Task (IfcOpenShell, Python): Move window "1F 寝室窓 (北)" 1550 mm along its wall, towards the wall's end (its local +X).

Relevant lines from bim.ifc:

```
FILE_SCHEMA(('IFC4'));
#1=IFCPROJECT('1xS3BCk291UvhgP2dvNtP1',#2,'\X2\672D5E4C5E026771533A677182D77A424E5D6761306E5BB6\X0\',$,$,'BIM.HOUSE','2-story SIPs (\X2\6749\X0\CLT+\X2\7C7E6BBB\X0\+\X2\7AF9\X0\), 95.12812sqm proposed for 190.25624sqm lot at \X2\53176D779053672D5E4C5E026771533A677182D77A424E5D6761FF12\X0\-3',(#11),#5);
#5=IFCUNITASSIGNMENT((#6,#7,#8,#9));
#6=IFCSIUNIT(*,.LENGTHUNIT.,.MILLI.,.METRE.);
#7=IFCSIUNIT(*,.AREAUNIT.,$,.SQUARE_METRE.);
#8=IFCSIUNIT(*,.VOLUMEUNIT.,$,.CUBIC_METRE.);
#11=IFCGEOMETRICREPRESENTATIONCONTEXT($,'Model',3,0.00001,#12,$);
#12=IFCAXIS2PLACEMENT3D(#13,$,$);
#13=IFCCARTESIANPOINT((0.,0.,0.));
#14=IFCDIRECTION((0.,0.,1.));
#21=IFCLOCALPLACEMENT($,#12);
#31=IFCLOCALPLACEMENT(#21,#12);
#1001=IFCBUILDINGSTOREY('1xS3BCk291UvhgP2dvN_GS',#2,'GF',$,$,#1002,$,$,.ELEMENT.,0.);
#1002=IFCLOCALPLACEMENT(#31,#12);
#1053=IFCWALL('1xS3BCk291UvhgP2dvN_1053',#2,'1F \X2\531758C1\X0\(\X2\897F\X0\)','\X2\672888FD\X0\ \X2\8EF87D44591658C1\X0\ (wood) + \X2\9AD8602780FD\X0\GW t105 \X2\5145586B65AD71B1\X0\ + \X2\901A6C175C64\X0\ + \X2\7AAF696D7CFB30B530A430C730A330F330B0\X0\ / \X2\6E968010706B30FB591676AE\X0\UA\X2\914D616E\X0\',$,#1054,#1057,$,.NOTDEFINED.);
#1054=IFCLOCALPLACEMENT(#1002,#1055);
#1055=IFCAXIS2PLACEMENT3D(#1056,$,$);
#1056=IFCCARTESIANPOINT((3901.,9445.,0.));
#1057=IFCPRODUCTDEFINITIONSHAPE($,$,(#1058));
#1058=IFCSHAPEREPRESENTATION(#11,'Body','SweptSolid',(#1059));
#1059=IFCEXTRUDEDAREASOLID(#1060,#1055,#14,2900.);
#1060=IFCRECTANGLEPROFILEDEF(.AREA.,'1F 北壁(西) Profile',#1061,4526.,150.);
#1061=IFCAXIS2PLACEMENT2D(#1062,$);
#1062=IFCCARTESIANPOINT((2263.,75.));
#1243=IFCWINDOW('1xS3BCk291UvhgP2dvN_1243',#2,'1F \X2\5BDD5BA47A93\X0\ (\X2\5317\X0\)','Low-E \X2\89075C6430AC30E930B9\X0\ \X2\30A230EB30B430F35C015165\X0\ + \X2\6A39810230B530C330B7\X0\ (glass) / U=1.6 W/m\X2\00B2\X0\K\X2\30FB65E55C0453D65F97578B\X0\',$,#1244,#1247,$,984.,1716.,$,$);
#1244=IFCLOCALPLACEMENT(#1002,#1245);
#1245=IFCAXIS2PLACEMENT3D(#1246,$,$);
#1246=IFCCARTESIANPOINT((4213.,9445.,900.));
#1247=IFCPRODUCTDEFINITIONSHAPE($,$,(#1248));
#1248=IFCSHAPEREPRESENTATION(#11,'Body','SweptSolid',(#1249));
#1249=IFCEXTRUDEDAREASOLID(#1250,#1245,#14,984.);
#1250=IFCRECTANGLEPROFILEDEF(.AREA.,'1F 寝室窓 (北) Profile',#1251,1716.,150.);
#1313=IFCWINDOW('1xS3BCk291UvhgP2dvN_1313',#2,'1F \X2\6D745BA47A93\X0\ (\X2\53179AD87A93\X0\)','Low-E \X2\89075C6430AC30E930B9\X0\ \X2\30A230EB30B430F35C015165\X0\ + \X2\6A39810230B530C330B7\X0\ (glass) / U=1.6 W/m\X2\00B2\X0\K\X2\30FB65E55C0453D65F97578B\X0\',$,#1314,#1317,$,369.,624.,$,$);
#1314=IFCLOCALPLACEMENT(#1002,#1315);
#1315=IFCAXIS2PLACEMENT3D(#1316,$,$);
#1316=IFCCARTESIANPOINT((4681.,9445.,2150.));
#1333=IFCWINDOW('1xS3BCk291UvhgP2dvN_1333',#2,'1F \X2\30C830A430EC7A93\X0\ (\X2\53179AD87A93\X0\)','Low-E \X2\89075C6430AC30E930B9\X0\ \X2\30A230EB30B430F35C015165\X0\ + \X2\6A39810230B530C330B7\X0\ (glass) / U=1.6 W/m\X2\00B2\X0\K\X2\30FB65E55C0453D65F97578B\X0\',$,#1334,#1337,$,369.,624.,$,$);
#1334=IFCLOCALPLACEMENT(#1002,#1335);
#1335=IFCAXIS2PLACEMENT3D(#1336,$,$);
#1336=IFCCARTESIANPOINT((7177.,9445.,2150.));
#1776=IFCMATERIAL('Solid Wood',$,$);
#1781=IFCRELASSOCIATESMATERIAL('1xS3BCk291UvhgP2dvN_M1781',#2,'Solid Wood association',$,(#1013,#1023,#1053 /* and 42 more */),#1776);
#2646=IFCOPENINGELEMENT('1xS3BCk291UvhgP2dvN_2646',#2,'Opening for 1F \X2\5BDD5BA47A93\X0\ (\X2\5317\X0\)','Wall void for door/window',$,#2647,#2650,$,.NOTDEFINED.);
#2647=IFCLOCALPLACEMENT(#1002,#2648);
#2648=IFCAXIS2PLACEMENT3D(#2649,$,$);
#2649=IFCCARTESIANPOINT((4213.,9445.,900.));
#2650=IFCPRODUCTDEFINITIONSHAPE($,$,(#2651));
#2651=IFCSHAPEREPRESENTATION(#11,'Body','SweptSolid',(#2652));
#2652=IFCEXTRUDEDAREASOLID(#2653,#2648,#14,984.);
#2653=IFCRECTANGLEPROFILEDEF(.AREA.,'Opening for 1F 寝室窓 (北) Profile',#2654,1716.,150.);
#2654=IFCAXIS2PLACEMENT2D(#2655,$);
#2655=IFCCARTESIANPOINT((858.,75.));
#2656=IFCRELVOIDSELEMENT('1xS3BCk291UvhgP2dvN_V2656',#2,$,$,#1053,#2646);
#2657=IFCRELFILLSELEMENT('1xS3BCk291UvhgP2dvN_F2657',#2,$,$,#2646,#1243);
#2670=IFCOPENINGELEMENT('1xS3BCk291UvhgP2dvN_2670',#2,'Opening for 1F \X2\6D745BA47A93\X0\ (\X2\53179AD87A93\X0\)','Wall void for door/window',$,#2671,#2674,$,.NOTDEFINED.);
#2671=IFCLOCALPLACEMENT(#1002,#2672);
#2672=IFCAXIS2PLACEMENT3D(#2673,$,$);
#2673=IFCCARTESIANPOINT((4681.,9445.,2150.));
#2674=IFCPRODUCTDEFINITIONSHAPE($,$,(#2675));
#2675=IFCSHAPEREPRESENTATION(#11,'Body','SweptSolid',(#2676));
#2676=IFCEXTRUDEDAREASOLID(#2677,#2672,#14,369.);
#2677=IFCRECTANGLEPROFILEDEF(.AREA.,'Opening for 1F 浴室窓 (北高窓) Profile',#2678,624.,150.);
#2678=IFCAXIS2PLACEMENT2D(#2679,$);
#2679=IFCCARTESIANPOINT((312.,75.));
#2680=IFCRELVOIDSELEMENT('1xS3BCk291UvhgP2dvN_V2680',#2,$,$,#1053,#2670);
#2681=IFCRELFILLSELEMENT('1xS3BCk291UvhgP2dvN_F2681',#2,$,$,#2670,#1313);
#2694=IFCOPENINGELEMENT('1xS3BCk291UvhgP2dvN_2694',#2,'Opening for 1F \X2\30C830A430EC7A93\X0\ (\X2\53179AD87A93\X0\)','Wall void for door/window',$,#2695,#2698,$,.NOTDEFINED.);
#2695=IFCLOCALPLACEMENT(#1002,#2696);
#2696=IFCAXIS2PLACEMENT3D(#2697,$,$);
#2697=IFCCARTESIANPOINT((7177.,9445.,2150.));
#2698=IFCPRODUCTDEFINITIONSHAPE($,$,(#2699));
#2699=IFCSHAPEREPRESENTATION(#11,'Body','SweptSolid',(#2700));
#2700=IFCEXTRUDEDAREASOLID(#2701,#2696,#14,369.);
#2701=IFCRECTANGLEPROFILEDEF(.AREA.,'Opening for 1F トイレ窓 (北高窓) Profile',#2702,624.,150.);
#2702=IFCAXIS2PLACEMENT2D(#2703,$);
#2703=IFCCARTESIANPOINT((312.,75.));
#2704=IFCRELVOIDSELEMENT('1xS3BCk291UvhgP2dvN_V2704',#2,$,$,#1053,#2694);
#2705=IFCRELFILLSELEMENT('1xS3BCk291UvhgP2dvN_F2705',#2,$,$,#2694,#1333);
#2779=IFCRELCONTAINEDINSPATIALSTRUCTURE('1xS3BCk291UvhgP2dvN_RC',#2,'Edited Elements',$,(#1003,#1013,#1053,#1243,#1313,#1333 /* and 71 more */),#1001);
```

```python
import ifcopenshell
import ifcopenshell.api.geometry
import ifcopenshell.util.placement

model = ifcopenshell.open("bim.ifc")

window = model.by_id(1243)
opening = window.FillsVoids[0].RelatingOpeningElement
wall = opening.VoidsElements[0].RelatingBuildingElement

wall_matrix = ifcopenshell.util.placement.get_local_placement(wall.ObjectPlacement)
shift = wall_matrix[:3, 0] * 1550.0
before = ifcopenshell.util.placement.get_local_placement(window.ObjectPlacement)[:3, 3].copy()

# The window is not placed relative to its opening, so move both.
for product in (opening, window):
    matrix = ifcopenshell.util.placement.get_local_placement(product.ObjectPlacement)
    matrix[:3, 3] += shift
    ifcopenshell.api.geometry.edit_object_placement(model, product=product, matrix=matrix, is_si=False)

after = ifcopenshell.util.placement.get_local_placement(window.ObjectPlacement)[:3, 3]
print("window moved by", (after - before).round(3) + 0.0)

model.write("bim_v2.ifc")
```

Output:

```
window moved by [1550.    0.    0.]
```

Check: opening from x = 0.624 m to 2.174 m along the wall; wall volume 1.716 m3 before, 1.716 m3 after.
